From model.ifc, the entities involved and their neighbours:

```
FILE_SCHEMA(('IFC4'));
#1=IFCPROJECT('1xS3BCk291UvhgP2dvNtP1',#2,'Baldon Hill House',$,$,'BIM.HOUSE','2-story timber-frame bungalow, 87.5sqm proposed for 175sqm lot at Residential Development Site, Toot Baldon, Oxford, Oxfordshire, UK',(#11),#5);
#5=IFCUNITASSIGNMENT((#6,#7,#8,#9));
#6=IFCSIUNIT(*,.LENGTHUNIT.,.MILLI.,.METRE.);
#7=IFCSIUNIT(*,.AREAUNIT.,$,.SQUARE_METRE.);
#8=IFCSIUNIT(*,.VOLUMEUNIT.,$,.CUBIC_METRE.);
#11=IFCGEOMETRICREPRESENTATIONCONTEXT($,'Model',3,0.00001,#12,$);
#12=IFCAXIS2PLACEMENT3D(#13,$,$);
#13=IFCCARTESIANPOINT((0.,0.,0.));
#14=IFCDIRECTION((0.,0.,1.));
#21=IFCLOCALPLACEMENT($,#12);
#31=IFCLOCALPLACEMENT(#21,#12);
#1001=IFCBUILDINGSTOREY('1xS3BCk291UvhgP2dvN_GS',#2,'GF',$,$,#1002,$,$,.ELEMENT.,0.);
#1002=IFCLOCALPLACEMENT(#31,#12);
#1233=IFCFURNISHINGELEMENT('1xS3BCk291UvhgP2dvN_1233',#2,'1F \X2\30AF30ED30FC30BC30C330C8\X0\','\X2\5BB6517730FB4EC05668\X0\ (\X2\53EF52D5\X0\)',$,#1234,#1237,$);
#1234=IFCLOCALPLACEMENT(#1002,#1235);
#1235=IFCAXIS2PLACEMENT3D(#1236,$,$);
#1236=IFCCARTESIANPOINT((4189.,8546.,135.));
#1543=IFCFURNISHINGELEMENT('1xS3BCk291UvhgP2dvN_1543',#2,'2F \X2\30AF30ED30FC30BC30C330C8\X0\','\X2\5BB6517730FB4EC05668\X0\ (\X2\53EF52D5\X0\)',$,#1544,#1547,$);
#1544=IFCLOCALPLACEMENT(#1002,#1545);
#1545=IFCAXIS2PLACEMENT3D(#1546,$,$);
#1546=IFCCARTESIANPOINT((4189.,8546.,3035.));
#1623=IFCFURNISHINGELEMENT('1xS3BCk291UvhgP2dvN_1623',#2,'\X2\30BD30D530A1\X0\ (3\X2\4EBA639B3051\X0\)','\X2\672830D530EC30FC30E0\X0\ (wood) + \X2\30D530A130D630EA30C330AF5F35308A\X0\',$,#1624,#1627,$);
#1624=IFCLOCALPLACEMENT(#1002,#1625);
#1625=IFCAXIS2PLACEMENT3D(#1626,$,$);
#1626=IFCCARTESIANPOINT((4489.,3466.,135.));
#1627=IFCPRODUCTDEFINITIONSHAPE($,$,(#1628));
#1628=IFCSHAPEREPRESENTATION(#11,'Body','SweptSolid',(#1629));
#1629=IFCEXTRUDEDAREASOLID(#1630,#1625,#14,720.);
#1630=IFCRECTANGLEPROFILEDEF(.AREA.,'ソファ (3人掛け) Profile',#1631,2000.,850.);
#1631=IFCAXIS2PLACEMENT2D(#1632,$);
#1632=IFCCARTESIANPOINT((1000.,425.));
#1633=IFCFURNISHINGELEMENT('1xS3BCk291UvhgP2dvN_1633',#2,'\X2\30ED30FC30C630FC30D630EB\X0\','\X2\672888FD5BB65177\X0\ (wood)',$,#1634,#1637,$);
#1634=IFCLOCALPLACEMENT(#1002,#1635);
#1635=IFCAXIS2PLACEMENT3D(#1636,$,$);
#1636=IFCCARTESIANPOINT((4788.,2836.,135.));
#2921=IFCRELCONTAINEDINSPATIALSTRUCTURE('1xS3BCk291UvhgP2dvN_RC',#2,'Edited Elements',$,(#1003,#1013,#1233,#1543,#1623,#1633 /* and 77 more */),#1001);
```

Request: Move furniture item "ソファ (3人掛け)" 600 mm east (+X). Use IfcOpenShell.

```python
import ifcopenshell
import ifcopenshell.api.geometry
import ifcopenshell.util.placement
import ifcopenshell.util.unit

model = ifcopenshell.open("model.ifc")
unit_scale = ifcopenshell.util.unit.calculate_unit_scale(model)

item = model.by_guid("1xS3BCk291UvhgP2dvN_1623")
matrix = ifcopenshell.util.placement.get_local_placement(item.ObjectPlacement)
matrix[0, 3] += 0.6 / unit_scale
ifcopenshell.api.geometry.edit_object_placement(model, product=item, matrix=matrix, is_si=False)

print(ifcopenshell.util.placement.get_local_placement(item.ObjectPlacement).round(3) + 0.0)

model.write("model_v2.ifc")
```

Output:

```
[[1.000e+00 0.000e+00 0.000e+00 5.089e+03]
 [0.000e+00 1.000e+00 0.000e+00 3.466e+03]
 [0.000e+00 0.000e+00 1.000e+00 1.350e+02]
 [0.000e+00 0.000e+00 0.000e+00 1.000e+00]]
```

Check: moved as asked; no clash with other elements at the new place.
